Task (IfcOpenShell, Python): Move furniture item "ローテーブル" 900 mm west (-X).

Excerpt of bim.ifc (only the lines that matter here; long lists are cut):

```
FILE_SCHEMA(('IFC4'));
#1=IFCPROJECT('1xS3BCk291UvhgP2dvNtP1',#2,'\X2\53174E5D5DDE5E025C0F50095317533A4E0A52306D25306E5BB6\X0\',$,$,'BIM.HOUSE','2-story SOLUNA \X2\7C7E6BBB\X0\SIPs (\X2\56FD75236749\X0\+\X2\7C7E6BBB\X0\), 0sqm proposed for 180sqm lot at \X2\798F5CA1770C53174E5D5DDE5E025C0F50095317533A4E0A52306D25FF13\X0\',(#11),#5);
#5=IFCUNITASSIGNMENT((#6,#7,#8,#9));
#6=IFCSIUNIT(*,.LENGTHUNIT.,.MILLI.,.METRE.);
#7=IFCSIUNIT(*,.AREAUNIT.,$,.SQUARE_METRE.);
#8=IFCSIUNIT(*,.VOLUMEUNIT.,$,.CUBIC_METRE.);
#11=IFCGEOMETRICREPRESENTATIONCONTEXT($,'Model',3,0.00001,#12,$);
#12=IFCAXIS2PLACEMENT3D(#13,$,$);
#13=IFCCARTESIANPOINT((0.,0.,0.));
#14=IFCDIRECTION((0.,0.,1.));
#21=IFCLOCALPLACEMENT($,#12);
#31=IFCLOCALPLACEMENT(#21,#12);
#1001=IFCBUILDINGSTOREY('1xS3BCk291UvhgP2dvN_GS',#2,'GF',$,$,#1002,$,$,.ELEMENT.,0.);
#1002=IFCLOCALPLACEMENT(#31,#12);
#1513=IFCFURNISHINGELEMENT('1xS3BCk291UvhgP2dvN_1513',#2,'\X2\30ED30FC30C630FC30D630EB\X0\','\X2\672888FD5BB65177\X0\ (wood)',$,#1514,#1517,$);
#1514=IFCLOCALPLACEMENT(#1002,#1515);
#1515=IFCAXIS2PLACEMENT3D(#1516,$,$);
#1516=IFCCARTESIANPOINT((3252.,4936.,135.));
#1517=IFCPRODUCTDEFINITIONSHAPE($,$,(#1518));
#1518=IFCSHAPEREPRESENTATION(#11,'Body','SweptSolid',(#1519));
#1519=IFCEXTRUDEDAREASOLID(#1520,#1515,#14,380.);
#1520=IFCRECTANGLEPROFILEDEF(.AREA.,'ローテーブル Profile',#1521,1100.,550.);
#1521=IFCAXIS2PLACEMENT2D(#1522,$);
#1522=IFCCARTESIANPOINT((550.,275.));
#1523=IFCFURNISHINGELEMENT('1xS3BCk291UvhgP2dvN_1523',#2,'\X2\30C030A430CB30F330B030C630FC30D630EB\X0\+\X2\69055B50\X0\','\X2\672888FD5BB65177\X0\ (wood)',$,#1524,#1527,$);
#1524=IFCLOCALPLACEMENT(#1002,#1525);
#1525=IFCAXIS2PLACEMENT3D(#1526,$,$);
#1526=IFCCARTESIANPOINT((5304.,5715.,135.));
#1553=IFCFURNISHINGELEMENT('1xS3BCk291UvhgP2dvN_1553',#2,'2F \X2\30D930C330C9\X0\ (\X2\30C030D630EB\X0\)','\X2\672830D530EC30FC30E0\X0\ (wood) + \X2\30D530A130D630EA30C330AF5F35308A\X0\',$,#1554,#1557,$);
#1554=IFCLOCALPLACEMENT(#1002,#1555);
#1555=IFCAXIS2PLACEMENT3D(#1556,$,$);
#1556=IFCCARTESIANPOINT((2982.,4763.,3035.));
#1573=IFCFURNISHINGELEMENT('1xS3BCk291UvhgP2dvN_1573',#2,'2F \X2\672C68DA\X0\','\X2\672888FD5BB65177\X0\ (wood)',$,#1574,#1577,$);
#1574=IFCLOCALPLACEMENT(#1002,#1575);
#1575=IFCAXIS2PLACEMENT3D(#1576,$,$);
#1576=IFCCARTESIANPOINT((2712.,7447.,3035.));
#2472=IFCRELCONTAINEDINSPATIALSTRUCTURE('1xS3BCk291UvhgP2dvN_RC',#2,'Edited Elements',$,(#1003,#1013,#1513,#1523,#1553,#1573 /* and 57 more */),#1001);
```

```python
import ifcopenshell
import ifcopenshell.api.geometry
import ifcopenshell.util.placement
import ifcopenshell.util.unit

model = ifcopenshell.open("bim.ifc")
unit_scale = ifcopenshell.util.unit.calculate_unit_scale(model)

item = model.by_guid("1xS3BCk291UvhgP2dvN_1513")
matrix = ifcopenshell.util.placement.get_local_placement(item.ObjectPlacement)
matrix[0, 3] -= 0.9 / unit_scale
ifcopenshell.api.geometry.edit_object_placement(model, product=item, matrix=matrix, is_si=False)

print(ifcopenshell.util.placement.get_local_placement(item.ObjectPlacement).round(3) + 0.0)

model.write("bim_updated.ifc")
```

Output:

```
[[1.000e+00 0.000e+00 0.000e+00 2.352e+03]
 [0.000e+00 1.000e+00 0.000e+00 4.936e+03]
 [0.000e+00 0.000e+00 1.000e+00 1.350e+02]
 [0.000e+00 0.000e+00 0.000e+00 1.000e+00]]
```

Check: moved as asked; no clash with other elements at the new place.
